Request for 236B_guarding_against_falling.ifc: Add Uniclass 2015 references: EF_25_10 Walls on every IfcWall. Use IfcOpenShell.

First a look at what the model holds.

```python
import ifcopenshell

model = ifcopenshell.open("236B_guarding_against_falling.ifc")
print(model.schema)
print("classifications:", [c.Name for c in model.by_type("IfcClassification")])
for ifc_class in ("IfcDoor", "IfcRoof", "IfcStair", "IfcWall", "IfcWindow"):
    print(ifc_class, len(model.by_type(ifc_class)))
```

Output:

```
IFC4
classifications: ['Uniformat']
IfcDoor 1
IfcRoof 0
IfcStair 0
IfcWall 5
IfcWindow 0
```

```python
import ifcopenshell
import ifcopenshell.api.classification

model = ifcopenshell.open("236B_guarding_against_falling.ifc")

system = ifcopenshell.api.classification.add_classification(model, classification="Uniclass 2015")

codes = {
    "IfcWall": ("EF_25_10", "Walls"),
}
for ifc_class, (code, name) in codes.items():
    products = model.by_type(ifc_class)
    ifcopenshell.api.classification.add_reference(
        model, products=products, classification=system, identification=code, name=name
    )
    print(code, len(products))

model.write("236B_guarding_against_falling_rev.ifc")
```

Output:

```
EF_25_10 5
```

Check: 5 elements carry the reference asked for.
